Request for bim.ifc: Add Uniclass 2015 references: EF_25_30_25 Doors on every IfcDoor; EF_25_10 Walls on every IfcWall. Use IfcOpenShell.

First a look at what the model holds.

```python
import ifcopenshell

model = ifcopenshell.open("bim.ifc")
print(model.schema)
print("classifications:", [c.Name for c in model.by_type("IfcClassification")])
for ifc_class in ("IfcDoor", "IfcRoof", "IfcStair", "IfcWall", "IfcWindow"):
    print(ifc_class, len(model.by_type(ifc_class)))
```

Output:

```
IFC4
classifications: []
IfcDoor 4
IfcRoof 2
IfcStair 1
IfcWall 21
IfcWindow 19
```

```python
import ifcopenshell
import ifcopenshell.api.classification

model = ifcopenshell.open("bim.ifc")

system = ifcopenshell.api.classification.add_classification(model, classification="Uniclass 2015")

codes = {
    "IfcDoor": ("EF_25_30_25", "Doors"),
    "IfcWall": ("EF_25_10", "Walls"),
}
for ifc_class, (code, name) in codes.items():
    products = model.by_type(ifc_class)
    ifcopenshell.api.classification.add_reference(
        model, products=products, classification=system, identification=code, name=name
    )
    print(code, len(products))

model.write("bim_rev.ifc")
```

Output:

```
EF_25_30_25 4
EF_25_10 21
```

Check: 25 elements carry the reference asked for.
